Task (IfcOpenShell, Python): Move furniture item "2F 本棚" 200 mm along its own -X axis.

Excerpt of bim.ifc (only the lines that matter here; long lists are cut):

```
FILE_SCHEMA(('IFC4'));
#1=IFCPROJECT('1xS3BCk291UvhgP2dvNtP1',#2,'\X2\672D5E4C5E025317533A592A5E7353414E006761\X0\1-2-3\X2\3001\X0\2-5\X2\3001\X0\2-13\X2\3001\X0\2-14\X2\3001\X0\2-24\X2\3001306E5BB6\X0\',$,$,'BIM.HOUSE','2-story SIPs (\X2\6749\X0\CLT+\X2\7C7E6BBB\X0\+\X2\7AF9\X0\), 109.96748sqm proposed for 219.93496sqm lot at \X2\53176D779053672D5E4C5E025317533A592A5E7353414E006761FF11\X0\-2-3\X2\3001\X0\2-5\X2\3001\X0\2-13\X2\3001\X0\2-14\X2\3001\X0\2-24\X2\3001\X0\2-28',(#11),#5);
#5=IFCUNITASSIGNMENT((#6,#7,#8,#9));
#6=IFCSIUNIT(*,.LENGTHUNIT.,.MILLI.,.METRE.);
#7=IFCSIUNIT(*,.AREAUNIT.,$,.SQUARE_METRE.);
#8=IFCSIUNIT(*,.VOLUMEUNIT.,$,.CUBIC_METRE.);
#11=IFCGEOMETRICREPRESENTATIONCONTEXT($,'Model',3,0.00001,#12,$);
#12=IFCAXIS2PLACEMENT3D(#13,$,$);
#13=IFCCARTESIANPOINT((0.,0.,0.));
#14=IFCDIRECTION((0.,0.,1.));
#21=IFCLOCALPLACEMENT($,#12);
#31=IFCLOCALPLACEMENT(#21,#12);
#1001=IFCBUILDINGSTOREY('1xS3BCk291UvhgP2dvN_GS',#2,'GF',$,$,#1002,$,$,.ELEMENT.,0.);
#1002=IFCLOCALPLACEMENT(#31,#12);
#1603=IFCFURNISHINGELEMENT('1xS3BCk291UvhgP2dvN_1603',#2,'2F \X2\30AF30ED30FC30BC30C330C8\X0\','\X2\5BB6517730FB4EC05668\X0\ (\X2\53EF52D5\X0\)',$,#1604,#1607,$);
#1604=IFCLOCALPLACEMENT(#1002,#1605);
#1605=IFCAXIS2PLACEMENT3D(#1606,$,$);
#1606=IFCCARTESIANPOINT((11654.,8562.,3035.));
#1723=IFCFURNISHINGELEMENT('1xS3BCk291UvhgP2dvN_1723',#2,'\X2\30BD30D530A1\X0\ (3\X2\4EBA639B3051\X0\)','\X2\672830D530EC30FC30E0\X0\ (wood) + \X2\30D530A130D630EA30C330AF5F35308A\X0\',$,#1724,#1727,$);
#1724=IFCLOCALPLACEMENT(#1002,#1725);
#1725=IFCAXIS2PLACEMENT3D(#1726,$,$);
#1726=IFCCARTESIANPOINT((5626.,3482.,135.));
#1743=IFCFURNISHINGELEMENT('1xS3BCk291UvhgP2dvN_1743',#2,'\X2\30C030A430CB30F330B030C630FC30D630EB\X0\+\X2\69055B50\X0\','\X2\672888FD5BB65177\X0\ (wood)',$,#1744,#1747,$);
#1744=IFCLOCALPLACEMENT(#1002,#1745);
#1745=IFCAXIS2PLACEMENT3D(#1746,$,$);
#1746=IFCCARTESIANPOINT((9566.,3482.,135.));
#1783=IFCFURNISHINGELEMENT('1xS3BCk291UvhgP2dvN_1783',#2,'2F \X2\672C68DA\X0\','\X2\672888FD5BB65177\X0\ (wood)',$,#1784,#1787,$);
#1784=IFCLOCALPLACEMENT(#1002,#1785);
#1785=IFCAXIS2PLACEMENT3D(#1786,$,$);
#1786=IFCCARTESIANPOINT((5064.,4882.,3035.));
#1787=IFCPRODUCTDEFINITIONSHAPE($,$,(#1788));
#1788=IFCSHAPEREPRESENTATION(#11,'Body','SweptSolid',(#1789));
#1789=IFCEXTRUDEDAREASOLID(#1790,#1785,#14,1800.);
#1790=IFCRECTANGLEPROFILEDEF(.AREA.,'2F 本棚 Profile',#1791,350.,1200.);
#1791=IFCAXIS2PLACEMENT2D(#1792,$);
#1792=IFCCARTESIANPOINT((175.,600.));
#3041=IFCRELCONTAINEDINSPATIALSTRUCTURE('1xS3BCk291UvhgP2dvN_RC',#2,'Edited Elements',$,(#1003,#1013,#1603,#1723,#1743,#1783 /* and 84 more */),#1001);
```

```python
import ifcopenshell
import ifcopenshell.api.geometry
import ifcopenshell.util.placement

model = ifcopenshell.open("bim.ifc")

item = model.by_guid("1xS3BCk291UvhgP2dvN_1783")
matrix = ifcopenshell.util.placement.get_local_placement(item.ObjectPlacement)
matrix[:3, 3] -= matrix[:3, 0] * 200.0
ifcopenshell.api.geometry.edit_object_placement(model, product=item, matrix=matrix, is_si=False)

print(ifcopenshell.util.placement.get_local_placement(item.ObjectPlacement).round(3) + 0.0)

model.write("bim_rev.ifc")
```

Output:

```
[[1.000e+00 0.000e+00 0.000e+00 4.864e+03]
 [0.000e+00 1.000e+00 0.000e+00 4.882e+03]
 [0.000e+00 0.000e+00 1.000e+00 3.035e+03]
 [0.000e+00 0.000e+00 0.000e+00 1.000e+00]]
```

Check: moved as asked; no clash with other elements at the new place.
